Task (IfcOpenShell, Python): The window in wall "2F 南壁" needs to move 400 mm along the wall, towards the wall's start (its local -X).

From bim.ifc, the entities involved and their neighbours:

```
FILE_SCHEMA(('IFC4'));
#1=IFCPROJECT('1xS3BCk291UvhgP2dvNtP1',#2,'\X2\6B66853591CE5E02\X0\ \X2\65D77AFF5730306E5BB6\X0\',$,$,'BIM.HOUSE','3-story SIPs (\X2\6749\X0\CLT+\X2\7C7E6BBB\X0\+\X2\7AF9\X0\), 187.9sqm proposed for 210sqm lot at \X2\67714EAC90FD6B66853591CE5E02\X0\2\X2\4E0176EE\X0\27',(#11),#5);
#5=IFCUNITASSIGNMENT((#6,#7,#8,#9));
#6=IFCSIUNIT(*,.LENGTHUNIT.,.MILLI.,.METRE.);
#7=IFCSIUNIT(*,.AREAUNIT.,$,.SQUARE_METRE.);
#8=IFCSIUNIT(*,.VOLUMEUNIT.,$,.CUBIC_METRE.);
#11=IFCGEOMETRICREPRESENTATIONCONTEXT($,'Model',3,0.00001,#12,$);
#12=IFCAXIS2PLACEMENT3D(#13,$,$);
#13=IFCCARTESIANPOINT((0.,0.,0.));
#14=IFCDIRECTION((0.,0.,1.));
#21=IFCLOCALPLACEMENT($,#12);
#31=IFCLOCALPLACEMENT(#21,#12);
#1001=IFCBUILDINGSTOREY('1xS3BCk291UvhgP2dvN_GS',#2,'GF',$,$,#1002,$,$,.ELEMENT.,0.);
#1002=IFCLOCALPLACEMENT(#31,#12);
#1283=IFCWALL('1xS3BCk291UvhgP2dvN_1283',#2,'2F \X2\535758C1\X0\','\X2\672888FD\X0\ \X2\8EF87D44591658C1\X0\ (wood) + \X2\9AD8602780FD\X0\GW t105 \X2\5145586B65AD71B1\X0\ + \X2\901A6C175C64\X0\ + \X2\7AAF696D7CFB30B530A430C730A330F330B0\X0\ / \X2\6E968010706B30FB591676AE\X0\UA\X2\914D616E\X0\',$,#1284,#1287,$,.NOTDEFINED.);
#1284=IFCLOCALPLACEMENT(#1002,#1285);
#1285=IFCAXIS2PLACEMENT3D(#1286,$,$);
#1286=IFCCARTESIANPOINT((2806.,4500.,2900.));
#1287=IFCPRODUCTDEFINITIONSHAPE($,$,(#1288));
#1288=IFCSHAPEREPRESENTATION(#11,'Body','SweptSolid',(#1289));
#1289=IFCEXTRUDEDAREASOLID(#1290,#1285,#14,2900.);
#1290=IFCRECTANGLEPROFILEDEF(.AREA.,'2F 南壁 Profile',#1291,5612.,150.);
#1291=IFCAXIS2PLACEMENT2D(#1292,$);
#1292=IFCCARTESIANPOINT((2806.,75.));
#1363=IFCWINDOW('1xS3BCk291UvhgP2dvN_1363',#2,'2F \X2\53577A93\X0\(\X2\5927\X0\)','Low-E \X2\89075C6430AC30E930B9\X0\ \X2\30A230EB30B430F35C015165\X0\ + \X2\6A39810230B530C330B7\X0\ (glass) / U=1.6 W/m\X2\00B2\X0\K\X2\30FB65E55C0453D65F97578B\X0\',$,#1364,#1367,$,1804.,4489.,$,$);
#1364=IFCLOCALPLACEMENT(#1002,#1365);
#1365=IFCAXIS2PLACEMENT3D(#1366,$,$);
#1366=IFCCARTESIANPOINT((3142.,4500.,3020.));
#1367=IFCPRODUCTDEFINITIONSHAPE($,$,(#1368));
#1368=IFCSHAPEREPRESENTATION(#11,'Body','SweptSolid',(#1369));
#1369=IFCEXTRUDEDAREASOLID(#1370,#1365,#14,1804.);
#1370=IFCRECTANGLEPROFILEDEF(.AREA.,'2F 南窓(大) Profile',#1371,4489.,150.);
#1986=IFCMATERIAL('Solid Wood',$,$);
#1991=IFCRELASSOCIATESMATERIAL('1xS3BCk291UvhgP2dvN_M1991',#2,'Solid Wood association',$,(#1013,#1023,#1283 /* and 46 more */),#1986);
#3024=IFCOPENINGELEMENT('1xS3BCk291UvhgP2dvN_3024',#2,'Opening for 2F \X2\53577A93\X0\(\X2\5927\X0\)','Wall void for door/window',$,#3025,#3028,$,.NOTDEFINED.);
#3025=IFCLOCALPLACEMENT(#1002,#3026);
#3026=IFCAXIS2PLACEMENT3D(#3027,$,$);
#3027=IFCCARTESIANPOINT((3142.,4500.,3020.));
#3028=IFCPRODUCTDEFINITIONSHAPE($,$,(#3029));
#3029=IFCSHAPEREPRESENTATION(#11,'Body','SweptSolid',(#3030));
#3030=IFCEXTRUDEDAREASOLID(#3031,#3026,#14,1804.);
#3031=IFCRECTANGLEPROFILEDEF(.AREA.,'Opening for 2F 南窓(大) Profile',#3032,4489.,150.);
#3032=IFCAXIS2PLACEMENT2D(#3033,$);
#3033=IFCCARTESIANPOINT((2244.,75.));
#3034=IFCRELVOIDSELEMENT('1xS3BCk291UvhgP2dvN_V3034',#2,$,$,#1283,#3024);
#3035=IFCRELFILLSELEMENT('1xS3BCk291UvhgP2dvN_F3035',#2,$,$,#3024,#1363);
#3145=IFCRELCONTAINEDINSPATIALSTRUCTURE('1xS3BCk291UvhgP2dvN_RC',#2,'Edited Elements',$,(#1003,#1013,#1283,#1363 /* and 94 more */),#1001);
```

```python
import ifcopenshell
import ifcopenshell.api.geometry
import ifcopenshell.util.placement

model = ifcopenshell.open("bim.ifc")

window = model.by_guid("1xS3BCk291UvhgP2dvN_1363")
opening = window.FillsVoids[0].RelatingOpeningElement
wall = opening.VoidsElements[0].RelatingBuildingElement

wall_matrix = ifcopenshell.util.placement.get_local_placement(wall.ObjectPlacement)
shift = wall_matrix[:3, 0] * -400.0
before = ifcopenshell.util.placement.get_local_placement(window.ObjectPlacement)[:3, 3].copy()

# The window is not placed relative to its opening, so move both.
for product in (opening, window):
    matrix = ifcopenshell.util.placement.get_local_placement(product.ObjectPlacement)
    matrix[:3, 3] += shift
    ifcopenshell.api.geometry.edit_object_placement(model, product=product, matrix=matrix, is_si=False)

after = ifcopenshell.util.placement.get_local_placement(window.ObjectPlacement)[:3, 3]
print("window moved by", (after - before).round(3) + 0.0)

model.write("bim_rev.ifc")
```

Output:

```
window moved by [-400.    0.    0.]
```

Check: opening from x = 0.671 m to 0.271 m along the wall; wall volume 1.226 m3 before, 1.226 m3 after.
